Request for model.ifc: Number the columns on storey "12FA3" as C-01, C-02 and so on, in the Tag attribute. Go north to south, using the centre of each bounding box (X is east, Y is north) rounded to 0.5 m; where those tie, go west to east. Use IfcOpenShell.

First a look at what the model holds.

```python
import ifcopenshell
import ifcopenshell.util.element
import ifcopenshell.util.placement

model = ifcopenshell.open("model.ifc")
print(model.schema)
storey = next(s for s in model.by_type("IfcBuildingStorey") if s.Name == "12FA3")
columns = [e for e in ifcopenshell.util.element.get_decomposition(storey) if e.is_a("IfcColumn")]
for e in sorted(columns, key=lambda e: e.id()):
    origin = ifcopenshell.util.placement.get_local_placement(e.ObjectPlacement)[:3, 3]
    print(e.id(), e.Tag, e.Name, origin.round(2) + 0.0, sep=" | ")
```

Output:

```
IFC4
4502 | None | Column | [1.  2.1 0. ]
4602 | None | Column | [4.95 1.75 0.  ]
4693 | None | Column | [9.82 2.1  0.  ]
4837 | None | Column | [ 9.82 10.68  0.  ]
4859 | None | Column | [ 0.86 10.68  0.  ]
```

```python
import ifcopenshell
import ifcopenshell.geom
import ifcopenshell.util.element
import ifcopenshell.util.shape

model = ifcopenshell.open("model.ifc")
settings = ifcopenshell.geom.settings()
settings.set("use-world-coords", True)


def centre(element):
    shape = ifcopenshell.geom.create_shape(settings, element)
    return ifcopenshell.util.shape.get_bbox_centroid(shape.geometry)


storey = next(s for s in model.by_type("IfcBuildingStorey") if s.Name == "12FA3")
columns = [e for e in ifcopenshell.util.element.get_decomposition(storey) if e.is_a("IfcColumn")]

# Insertion points can sit at a corner or the storey origin, so sort by the geometry (in metres).
centres = {e: centre(e) for e in columns}
columns.sort(key=lambda e: (-round(centres[e][1] / 0.5), centres[e][0]))

for i, e in enumerate(columns, start=1):
    number = f"C-{i:02d}"
    e.Tag = number
    print(e.id(), number)

model.write("model-out.ifc")
```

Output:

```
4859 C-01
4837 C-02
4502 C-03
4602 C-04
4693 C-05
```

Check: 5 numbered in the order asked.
